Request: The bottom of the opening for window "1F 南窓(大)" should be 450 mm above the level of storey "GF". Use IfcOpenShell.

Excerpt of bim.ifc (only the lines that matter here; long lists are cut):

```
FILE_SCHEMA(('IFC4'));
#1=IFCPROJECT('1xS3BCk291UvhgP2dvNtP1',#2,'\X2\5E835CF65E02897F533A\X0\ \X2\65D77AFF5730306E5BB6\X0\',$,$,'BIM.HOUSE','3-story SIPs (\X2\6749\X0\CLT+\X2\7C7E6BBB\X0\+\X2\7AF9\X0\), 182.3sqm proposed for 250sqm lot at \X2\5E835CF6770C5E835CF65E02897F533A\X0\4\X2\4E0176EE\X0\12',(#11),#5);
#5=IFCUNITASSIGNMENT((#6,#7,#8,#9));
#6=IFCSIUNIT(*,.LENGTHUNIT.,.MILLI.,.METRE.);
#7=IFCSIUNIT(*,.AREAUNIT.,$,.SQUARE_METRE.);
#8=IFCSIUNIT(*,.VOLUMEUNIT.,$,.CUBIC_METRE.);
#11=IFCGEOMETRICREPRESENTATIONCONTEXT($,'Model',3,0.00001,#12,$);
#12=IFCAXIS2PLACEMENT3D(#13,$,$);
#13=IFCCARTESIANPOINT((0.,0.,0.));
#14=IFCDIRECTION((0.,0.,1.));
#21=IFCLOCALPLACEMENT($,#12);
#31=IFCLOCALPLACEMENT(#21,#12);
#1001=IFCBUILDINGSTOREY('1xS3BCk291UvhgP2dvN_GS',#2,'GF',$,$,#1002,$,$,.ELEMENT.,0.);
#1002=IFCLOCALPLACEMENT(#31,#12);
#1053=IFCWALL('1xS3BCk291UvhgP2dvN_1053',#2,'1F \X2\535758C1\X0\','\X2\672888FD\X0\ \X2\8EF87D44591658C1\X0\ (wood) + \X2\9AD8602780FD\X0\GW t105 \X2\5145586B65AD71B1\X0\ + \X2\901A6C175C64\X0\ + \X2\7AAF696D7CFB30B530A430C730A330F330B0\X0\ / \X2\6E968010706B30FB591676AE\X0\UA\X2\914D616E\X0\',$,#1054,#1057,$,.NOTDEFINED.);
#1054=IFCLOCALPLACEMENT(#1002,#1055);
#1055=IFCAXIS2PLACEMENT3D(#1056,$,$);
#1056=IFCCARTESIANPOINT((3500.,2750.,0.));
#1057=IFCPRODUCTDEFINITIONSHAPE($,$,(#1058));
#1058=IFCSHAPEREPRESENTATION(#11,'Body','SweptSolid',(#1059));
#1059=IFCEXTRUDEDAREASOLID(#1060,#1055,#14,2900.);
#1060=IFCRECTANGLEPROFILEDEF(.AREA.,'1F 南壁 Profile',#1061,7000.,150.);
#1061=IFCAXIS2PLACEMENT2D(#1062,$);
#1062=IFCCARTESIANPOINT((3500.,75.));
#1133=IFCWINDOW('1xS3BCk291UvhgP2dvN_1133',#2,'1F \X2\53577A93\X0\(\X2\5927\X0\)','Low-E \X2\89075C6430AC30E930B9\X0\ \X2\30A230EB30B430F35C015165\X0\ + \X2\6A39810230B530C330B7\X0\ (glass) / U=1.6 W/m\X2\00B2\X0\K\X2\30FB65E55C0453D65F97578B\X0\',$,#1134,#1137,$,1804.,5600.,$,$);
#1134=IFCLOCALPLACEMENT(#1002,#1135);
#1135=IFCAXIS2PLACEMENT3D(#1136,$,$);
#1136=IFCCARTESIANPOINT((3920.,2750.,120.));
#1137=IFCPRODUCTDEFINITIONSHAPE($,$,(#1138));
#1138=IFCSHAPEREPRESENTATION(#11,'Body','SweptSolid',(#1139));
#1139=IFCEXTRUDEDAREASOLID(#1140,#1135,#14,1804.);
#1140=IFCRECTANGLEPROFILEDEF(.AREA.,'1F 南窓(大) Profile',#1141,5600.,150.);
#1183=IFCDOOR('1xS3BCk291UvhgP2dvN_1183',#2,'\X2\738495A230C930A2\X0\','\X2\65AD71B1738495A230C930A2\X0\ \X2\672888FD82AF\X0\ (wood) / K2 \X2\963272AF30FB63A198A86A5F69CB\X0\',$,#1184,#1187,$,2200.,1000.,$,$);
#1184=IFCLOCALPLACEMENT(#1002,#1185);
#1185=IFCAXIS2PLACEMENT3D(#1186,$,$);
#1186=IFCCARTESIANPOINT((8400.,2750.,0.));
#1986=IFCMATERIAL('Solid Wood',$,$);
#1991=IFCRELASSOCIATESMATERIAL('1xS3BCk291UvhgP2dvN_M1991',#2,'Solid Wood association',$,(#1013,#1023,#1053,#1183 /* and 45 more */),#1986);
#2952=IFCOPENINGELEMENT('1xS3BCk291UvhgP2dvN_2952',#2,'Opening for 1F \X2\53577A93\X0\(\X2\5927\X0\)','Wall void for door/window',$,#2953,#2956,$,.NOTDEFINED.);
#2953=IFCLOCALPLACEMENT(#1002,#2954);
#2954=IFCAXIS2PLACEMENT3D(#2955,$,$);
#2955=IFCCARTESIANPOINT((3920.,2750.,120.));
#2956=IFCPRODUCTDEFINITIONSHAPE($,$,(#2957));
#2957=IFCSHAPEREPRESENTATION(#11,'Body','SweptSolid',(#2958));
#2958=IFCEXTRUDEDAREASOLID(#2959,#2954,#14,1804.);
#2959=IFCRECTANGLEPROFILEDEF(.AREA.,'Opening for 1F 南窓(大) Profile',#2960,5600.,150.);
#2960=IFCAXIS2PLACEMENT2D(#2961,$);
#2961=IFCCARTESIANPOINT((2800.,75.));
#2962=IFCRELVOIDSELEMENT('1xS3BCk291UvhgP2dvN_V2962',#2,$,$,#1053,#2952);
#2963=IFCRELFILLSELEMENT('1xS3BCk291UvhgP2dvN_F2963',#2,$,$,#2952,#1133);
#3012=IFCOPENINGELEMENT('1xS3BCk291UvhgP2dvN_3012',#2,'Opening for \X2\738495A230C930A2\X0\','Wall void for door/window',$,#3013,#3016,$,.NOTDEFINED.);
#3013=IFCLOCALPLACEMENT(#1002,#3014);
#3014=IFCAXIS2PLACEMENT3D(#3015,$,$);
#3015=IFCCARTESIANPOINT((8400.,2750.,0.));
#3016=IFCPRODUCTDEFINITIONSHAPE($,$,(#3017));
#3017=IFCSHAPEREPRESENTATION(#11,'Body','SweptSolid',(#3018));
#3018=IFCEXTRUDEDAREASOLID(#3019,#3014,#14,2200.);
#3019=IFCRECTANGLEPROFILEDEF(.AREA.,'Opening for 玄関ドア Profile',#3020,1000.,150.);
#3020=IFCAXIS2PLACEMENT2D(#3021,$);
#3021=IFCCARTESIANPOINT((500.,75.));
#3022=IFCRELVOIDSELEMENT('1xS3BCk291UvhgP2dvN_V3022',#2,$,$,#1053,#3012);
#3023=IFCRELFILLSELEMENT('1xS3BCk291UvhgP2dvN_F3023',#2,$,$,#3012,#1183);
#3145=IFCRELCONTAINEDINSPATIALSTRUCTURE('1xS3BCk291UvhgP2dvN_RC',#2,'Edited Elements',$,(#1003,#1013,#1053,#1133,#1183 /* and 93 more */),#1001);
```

```python
import numpy as np
import ifcopenshell
import ifcopenshell.api.geometry
import ifcopenshell.geom
import ifcopenshell.util.element
import ifcopenshell.util.placement
import ifcopenshell.util.shape
import ifcopenshell.util.unit

model = ifcopenshell.open("bim.ifc")
unit_scale = ifcopenshell.util.unit.calculate_unit_scale(model)

window = model.by_guid("1xS3BCk291UvhgP2dvN_1133")
opening = window.FillsVoids[0].RelatingOpeningElement
storey = ifcopenshell.util.element.get_container(window, ifc_class="IfcBuildingStorey")
level = ifcopenshell.util.placement.get_local_placement(storey.ObjectPlacement)[2, 3]

# The opening's origin need not be at the sill, so measure its lowest point.
shape = ifcopenshell.geom.create_shape(ifcopenshell.geom.settings(), opening)
bottom = ifcopenshell.util.shape.get_shape_bottom_elevation(shape, shape.geometry) / unit_scale
dz = level + 0.45 / unit_scale - bottom

shift = np.array([0.0, 0.0, dz])
# The window is not placed relative to its opening, so move both.
for product in (opening, window):
    matrix = ifcopenshell.util.placement.get_local_placement(product.ObjectPlacement)
    matrix[:3, 3] += shift
    ifcopenshell.api.geometry.edit_object_placement(model, product=product, matrix=matrix, is_si=False)

print(f"moved by {dz * unit_scale:+.3f} m")

model.write("bim_edited.ifc")
```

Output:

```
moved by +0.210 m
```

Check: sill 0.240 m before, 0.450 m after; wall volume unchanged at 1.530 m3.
